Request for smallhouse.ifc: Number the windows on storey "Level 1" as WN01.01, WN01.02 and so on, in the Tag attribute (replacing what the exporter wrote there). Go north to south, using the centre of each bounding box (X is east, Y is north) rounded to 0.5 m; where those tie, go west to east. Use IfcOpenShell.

First a look at what the model holds.

```python
import ifcopenshell
import ifcopenshell.util.element
import ifcopenshell.util.placement

model = ifcopenshell.open("smallhouse.ifc")
print(model.schema)
storey = next(s for s in model.by_type("IfcBuildingStorey") if s.Name == "Level 1")
windows = [e for e in ifcopenshell.util.element.get_decomposition(storey) if e.is_a("IfcWindow")]
for e in sorted(windows, key=lambda e: e.id()):
    origin = ifcopenshell.util.placement.get_local_placement(e.ObjectPlacement)[:3, 3]
    print(e.id(), e.Tag, e.Name, origin.round(2) + 0.0, sep=" | ")
```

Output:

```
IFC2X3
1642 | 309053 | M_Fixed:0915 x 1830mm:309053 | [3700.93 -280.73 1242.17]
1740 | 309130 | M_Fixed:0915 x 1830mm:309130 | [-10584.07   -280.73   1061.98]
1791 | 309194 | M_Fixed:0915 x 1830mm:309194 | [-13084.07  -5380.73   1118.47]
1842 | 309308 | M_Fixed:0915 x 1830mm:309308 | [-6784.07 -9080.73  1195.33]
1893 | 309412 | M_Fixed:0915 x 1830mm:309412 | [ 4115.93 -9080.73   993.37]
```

```python
import ifcopenshell
import ifcopenshell.geom
import ifcopenshell.util.element
import ifcopenshell.util.shape

model = ifcopenshell.open("smallhouse.ifc")
settings = ifcopenshell.geom.settings()
settings.set("use-world-coords", True)


def centre(element):
    shape = ifcopenshell.geom.create_shape(settings, element)
    return ifcopenshell.util.shape.get_bbox_centroid(shape.geometry)


storey = next(s for s in model.by_type("IfcBuildingStorey") if s.Name == "Level 1")
windows = [e for e in ifcopenshell.util.element.get_decomposition(storey) if e.is_a("IfcWindow")]

# Insertion points can sit at a corner or the storey origin, so sort by the geometry (in metres).
centres = {e: centre(e) for e in windows}
windows.sort(key=lambda e: (-round(centres[e][1] / 0.5), centres[e][0]))

for i, e in enumerate(windows, start=1):
    number = f"WN01.{i:02d}"
    e.Tag = number
    print(e.id(), number)

model.write("smallhouse_edited.ifc")
```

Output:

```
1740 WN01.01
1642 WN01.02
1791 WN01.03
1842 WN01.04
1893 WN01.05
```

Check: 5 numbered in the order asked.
